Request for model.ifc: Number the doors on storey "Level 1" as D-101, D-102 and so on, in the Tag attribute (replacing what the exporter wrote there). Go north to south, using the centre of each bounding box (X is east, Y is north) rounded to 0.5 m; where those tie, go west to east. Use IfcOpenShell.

First a look at what the model holds.

```python
import ifcopenshell
import ifcopenshell.util.element
import ifcopenshell.util.placement

model = ifcopenshell.open("model.ifc")
print(model.schema)
storey = next(s for s in model.by_type("IfcBuildingStorey") if s.Name == "Level 1")
doors = [e for e in ifcopenshell.util.element.get_decomposition(storey) if e.is_a("IfcDoor")]
for e in sorted(doors, key=lambda e: e.id()):
    origin = ifcopenshell.util.placement.get_local_placement(e.ObjectPlacement)[:3, 3]
    print(e.id(), e.Tag, e.Name, origin.round(2) + 0.0, sep=" | ")
```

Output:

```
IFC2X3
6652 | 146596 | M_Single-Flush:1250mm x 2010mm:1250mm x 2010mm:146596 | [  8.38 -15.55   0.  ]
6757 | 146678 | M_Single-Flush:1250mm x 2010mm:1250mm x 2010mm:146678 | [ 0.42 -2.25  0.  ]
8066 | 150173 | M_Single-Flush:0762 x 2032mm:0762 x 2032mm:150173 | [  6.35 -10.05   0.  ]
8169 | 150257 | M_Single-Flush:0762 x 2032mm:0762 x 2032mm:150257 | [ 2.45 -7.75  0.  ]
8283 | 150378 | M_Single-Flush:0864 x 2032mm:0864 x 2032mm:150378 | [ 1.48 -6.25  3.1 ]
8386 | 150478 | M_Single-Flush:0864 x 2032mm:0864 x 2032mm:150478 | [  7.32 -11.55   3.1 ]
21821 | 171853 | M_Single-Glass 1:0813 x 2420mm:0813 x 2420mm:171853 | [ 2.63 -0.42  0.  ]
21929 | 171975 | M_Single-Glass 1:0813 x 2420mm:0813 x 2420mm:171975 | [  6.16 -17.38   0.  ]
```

```python
import ifcopenshell
import ifcopenshell.geom
import ifcopenshell.util.element
import ifcopenshell.util.shape

model = ifcopenshell.open("model.ifc")
settings = ifcopenshell.geom.settings()
settings.set("use-world-coords", True)


def centre(element):
    shape = ifcopenshell.geom.create_shape(settings, element)
    return ifcopenshell.util.shape.get_bbox_centroid(shape.geometry)


storey = next(s for s in model.by_type("IfcBuildingStorey") if s.Name == "Level 1")
doors = [e for e in ifcopenshell.util.element.get_decomposition(storey) if e.is_a("IfcDoor")]

# Insertion points can sit at a corner or the storey origin, so sort by the geometry (in metres).
centres = {e: centre(e) for e in doors}
doors.sort(key=lambda e: (-round(centres[e][1] / 0.5), centres[e][0]))

for i, e in enumerate(doors, start=1):
    number = f"D-1{i:02d}"
    e.Tag = number
    print(e.id(), number)

model.write("model_v2.ifc")
```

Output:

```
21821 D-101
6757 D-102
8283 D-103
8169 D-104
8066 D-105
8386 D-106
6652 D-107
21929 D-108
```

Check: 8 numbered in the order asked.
